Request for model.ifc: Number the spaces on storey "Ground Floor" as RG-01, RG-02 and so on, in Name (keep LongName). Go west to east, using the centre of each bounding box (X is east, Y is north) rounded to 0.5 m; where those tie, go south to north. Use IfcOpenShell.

First a look at what the model holds.

```python
import ifcopenshell
import ifcopenshell.util.element
import ifcopenshell.util.placement

model = ifcopenshell.open("model.ifc")
print(model.schema)
storey = next(s for s in model.by_type("IfcBuildingStorey") if s.Name == "Ground Floor")
spaces = [e for e in ifcopenshell.util.element.get_decomposition(storey) if e.is_a("IfcSpace")]
for e in sorted(spaces, key=lambda e: e.id()):
    origin = ifcopenshell.util.placement.get_local_placement(e.ObjectPlacement)[:3, 3]
    print(e.id(), e.Name, e.LongName, origin.round(2) + 0.0, sep=" | ")
```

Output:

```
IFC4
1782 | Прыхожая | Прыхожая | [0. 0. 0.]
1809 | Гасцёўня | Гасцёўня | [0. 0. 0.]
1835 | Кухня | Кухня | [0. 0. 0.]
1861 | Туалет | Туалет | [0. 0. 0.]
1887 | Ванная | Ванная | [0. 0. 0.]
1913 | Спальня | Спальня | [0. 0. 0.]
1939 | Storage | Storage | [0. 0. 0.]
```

```python
import ifcopenshell
import ifcopenshell.geom
import ifcopenshell.util.element
import ifcopenshell.util.shape

model = ifcopenshell.open("model.ifc")
settings = ifcopenshell.geom.settings()
settings.set("use-world-coords", True)


def centre(element):
    shape = ifcopenshell.geom.create_shape(settings, element)
    return ifcopenshell.util.shape.get_bbox_centroid(shape.geometry)


storey = next(s for s in model.by_type("IfcBuildingStorey") if s.Name == "Ground Floor")
spaces = [e for e in ifcopenshell.util.element.get_decomposition(storey) if e.is_a("IfcSpace")]

# Insertion points can sit at a corner or the storey origin, so sort by the geometry (in metres).
centres = {e: centre(e) for e in spaces}
spaces.sort(key=lambda e: (round(centres[e][0] / 0.5), centres[e][1]))

for i, e in enumerate(spaces, start=1):
    number = f"RG-{i:02d}"
    e.Name = number
    print(e.id(), number)

model.write("model_rev.ifc")
```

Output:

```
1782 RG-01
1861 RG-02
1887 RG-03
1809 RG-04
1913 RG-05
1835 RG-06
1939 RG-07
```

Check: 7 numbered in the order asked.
